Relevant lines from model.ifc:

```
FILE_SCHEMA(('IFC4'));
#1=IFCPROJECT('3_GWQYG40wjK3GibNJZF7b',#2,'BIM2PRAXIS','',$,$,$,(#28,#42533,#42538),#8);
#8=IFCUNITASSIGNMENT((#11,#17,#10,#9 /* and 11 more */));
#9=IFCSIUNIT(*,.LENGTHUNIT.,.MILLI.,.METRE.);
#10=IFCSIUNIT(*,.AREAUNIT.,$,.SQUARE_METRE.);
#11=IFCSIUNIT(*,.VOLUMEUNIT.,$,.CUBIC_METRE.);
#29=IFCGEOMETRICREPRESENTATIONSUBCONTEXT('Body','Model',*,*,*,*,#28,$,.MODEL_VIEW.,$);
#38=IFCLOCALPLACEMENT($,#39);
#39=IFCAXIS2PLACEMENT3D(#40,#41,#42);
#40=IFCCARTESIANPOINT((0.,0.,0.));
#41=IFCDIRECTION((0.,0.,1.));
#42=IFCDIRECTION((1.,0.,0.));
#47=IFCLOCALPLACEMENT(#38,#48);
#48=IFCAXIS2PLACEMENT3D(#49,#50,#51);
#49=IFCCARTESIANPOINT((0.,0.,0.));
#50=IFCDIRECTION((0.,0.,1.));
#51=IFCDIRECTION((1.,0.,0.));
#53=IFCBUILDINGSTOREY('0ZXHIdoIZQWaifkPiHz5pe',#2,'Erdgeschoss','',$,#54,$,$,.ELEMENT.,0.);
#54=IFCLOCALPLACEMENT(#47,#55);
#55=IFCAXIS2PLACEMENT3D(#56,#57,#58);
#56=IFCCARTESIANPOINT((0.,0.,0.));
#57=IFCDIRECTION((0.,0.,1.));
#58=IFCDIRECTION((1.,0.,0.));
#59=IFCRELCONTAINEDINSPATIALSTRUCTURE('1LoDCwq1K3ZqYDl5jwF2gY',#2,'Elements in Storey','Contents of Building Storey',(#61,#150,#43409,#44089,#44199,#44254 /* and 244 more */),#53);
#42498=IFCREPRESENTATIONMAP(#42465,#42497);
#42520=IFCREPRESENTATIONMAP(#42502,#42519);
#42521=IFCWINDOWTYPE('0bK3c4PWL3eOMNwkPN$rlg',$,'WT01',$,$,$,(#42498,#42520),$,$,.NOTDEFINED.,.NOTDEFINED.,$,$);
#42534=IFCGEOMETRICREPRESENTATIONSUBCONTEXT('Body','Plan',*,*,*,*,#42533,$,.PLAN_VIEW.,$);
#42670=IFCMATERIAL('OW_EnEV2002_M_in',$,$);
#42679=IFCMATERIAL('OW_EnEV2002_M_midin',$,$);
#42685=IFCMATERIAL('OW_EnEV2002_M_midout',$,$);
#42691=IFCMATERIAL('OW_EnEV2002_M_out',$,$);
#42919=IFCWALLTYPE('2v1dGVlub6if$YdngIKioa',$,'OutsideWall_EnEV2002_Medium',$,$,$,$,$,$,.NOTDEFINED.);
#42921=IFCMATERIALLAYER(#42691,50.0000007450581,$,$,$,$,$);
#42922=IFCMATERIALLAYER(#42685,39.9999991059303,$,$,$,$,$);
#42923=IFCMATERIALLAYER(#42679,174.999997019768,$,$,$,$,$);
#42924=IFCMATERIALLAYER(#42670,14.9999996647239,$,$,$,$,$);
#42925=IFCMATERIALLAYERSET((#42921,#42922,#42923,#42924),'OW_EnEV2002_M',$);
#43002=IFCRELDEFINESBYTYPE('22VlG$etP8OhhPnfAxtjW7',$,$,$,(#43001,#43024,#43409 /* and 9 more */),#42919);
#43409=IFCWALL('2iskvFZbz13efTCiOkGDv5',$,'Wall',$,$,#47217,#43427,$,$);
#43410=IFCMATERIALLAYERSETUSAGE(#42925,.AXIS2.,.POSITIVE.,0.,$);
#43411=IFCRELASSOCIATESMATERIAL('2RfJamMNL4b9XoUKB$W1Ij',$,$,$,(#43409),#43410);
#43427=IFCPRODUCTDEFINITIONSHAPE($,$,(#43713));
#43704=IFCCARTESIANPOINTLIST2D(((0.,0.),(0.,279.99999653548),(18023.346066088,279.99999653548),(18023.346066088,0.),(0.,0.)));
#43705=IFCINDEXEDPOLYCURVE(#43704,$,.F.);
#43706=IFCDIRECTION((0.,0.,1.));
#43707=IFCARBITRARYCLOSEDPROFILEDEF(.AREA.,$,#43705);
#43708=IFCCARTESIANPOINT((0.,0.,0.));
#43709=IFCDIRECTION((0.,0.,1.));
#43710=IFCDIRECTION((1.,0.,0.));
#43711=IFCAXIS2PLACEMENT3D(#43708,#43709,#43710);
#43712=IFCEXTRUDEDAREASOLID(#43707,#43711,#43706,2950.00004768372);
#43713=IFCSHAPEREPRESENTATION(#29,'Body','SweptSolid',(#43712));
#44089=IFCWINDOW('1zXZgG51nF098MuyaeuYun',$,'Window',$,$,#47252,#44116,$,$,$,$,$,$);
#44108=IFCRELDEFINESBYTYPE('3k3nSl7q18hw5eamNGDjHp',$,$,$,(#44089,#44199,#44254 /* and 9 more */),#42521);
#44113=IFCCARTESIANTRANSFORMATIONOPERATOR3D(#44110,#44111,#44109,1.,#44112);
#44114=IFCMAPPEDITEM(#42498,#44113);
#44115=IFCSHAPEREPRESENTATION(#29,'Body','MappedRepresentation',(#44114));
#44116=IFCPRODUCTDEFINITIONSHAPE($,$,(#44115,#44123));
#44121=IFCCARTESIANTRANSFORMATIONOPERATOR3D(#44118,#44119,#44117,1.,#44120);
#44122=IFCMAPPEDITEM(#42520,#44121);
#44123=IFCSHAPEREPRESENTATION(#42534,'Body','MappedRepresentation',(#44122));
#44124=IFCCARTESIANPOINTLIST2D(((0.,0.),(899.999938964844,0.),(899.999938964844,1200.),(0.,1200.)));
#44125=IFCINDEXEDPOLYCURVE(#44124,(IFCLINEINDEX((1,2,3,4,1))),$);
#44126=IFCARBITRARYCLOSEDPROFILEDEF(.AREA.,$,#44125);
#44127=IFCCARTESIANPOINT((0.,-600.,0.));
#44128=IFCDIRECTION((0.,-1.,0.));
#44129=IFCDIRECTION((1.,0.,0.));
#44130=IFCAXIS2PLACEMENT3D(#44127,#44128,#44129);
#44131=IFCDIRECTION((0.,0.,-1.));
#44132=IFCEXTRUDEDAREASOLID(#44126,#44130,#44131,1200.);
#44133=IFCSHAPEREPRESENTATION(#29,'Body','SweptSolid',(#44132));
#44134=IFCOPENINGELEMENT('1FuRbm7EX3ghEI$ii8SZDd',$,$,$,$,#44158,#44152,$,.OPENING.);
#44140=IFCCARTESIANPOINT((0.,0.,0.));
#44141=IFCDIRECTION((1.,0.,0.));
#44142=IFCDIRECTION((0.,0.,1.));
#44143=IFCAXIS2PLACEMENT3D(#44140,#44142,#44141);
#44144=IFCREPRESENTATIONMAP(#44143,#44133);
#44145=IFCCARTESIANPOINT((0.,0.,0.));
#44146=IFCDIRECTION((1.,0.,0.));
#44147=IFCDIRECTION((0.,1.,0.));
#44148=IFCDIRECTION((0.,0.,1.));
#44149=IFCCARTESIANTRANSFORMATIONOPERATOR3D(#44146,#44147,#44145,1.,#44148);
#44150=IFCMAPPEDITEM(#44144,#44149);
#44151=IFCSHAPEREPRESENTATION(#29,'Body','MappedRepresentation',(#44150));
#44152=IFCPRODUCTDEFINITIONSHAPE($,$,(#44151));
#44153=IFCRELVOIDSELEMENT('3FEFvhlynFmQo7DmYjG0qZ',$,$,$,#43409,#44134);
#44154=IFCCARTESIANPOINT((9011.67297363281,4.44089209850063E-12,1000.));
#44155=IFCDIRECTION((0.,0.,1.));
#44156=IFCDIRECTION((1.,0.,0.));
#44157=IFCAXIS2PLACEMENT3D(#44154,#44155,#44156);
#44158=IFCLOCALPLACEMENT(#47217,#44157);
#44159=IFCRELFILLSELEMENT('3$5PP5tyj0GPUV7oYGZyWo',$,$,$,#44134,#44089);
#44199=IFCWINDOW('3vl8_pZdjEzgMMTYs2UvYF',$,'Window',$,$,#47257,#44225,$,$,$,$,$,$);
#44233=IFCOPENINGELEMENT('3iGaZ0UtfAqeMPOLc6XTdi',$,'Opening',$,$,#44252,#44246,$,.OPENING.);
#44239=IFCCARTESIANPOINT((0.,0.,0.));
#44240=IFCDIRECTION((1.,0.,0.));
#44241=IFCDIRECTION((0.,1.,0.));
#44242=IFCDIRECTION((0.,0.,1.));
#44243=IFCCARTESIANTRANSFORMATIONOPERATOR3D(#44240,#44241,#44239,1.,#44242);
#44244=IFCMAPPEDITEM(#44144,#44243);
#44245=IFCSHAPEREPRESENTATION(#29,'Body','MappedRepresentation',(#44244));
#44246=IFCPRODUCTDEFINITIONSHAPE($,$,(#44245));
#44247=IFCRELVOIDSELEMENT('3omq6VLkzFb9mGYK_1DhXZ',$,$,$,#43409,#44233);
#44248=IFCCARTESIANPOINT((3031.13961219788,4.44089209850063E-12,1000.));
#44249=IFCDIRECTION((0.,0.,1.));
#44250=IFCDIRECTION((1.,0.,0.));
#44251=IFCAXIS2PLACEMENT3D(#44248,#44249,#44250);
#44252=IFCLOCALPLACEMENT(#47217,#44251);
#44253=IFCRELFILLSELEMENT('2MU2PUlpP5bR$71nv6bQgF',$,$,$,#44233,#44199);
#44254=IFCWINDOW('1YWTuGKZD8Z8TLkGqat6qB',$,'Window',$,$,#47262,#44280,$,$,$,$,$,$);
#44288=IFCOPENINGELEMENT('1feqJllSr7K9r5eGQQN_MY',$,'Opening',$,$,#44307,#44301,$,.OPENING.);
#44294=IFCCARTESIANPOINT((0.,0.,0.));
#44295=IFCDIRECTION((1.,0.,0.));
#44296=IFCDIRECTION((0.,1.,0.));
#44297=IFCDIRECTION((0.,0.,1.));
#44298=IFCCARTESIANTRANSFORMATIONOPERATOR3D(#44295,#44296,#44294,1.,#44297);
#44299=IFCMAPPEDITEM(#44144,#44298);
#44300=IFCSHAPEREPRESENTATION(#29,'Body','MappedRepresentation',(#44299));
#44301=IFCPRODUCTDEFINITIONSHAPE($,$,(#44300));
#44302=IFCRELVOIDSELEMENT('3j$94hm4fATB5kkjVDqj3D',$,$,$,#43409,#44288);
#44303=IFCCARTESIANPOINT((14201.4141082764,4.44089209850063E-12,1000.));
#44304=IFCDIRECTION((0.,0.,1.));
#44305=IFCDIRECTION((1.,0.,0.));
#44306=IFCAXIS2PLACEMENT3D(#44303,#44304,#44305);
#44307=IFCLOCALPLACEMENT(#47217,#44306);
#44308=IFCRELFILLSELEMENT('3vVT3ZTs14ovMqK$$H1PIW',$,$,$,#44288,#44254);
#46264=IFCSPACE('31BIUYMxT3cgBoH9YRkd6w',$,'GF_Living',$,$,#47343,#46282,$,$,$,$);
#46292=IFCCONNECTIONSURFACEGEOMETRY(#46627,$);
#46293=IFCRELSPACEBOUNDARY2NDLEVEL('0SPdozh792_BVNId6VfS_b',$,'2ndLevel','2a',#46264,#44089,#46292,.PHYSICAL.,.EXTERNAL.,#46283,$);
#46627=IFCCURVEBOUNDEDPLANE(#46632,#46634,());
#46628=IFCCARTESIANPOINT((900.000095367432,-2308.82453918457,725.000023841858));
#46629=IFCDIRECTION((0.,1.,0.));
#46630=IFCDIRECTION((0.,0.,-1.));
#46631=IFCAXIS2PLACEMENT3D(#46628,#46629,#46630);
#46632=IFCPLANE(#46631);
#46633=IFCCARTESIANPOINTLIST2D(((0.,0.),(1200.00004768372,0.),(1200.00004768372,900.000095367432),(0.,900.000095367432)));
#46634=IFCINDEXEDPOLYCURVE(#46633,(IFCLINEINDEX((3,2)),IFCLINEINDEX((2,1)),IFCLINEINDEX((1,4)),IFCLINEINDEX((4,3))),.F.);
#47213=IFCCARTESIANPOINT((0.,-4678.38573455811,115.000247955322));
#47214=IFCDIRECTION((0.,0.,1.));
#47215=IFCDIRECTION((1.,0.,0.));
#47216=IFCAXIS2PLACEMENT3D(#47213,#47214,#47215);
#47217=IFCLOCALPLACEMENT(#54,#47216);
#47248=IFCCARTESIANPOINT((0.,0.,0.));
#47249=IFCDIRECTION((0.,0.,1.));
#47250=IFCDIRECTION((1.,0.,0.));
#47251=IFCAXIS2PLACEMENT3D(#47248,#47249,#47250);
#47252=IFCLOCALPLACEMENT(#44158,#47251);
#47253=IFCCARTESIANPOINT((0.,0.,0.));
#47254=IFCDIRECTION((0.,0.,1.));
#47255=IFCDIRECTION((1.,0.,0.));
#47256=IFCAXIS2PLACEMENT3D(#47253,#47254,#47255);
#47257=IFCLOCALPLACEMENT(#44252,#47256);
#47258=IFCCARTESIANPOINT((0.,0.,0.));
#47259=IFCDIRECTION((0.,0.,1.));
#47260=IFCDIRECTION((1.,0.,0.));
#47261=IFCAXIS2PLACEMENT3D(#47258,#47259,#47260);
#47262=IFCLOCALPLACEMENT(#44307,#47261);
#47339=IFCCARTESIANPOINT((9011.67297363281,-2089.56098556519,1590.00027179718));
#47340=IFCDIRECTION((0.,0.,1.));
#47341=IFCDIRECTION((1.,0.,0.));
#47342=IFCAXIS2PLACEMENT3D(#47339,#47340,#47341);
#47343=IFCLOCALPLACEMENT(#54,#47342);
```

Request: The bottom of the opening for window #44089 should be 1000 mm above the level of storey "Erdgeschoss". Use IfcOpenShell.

```python
import numpy as np
import ifcopenshell
import ifcopenshell.api.geometry
import ifcopenshell.geom
import ifcopenshell.util.element
import ifcopenshell.util.placement
import ifcopenshell.util.shape
import ifcopenshell.util.unit

model = ifcopenshell.open("model.ifc")
unit_scale = ifcopenshell.util.unit.calculate_unit_scale(model)

window = model.by_guid("1zXZgG51nF098MuyaeuYun")
opening = window.FillsVoids[0].RelatingOpeningElement
storey = ifcopenshell.util.element.get_container(window, ifc_class="IfcBuildingStorey")
level = ifcopenshell.util.placement.get_local_placement(storey.ObjectPlacement)[2, 3]

# The opening's origin need not be at the sill, so measure its lowest point.
shape = ifcopenshell.geom.create_shape(ifcopenshell.geom.settings(), opening)
bottom = ifcopenshell.util.shape.get_shape_bottom_elevation(shape, shape.geometry) / unit_scale
dz = level + 1 / unit_scale - bottom

shift = np.array([0.0, 0.0, dz])
# The window is placed relative to its opening, so it follows when the opening moves.
matrix = ifcopenshell.util.placement.get_local_placement(opening.ObjectPlacement)
matrix[:3, 3] += shift
ifcopenshell.api.geometry.edit_object_placement(
    model, product=opening, matrix=matrix, is_si=False, should_transform_children=True
)

# Space boundary surfaces are stored in each space's coordinates; move them too.
for rel in window.ProvidesBoundaries:
    if not rel.ConnectionGeometry:
        continue
    surface = rel.ConnectionGeometry.SurfaceOnRelatingElement.BasisSurface
    space_matrix = ifcopenshell.util.placement.get_local_placement(rel.RelatingSpace.ObjectPlacement)
    point = np.array(surface.Position.Location.Coordinates) + space_matrix[:3, :3].T @ shift
    surface.Position = model.createIfcAxis2Placement3D(
        model.createIfcCartesianPoint(point.tolist()), surface.Position.Axis, surface.Position.RefDirection
    )

print(f"moved by {dz * unit_scale:+.3f} m")

model.write("model-out.ifc")
```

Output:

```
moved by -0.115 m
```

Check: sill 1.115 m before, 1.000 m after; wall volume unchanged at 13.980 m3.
